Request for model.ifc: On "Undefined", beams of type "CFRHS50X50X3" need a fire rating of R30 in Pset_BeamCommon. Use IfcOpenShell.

First a look at what the model holds.

```python
import ifcopenshell
import ifcopenshell.util.element

model = ifcopenshell.open("model.ifc")
print(model.schema)
storey = next(s for s in model.by_type("IfcBuildingStorey") if s.Name == "Undefined")
beams = [e for e in ifcopenshell.util.element.get_decomposition(storey) if e.is_a("IfcBeam")]
seen = {}
for e in beams:
    element_type = ifcopenshell.util.element.get_type(e)
    key = (element_type.Name if element_type != e and element_type else None, ifcopenshell.util.element.get_pset(e, "Pset_BeamCommon", "FireRating"))
    seen[key] = seen.get(key, 0) + 1
for (name, value), count in sorted(seen.items(), key=str):
    print(count, "x", name, "|", value)
```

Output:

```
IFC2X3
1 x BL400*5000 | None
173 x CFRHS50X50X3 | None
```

```python
import ifcopenshell
import ifcopenshell.api.pset
import ifcopenshell.util.element

model = ifcopenshell.open("model.ifc")

storey = next(s for s in model.by_type("IfcBuildingStorey") if s.Name == "Undefined")
beams = [e for e in ifcopenshell.util.element.get_decomposition(storey) if e.is_a("IfcBeam")]

count = 0
for e in beams:
    element_type = ifcopenshell.util.element.get_type(e)
    if element_type in (None, e) or element_type.Name != "CFRHS50X50X3":
        continue
    found = ifcopenshell.util.element.get_pset(e, "Pset_BeamCommon", should_inherit=False)
    if found:
        pset = model.by_id(found["id"])
        if len(ifcopenshell.util.element.get_elements_by_pset(pset)) > 1:
            pset = ifcopenshell.api.pset.unshare_pset(model, products=[e], pset=pset)[0]
    else:
        pset = ifcopenshell.api.pset.add_pset(model, product=e, name="Pset_BeamCommon")
    ifcopenshell.api.pset.edit_pset(model, pset=pset, properties={"FireRating": "R30"})
    count += 1

print(count, "beams updated")

model.write("model-out.ifc")
```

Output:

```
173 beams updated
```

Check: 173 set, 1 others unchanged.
